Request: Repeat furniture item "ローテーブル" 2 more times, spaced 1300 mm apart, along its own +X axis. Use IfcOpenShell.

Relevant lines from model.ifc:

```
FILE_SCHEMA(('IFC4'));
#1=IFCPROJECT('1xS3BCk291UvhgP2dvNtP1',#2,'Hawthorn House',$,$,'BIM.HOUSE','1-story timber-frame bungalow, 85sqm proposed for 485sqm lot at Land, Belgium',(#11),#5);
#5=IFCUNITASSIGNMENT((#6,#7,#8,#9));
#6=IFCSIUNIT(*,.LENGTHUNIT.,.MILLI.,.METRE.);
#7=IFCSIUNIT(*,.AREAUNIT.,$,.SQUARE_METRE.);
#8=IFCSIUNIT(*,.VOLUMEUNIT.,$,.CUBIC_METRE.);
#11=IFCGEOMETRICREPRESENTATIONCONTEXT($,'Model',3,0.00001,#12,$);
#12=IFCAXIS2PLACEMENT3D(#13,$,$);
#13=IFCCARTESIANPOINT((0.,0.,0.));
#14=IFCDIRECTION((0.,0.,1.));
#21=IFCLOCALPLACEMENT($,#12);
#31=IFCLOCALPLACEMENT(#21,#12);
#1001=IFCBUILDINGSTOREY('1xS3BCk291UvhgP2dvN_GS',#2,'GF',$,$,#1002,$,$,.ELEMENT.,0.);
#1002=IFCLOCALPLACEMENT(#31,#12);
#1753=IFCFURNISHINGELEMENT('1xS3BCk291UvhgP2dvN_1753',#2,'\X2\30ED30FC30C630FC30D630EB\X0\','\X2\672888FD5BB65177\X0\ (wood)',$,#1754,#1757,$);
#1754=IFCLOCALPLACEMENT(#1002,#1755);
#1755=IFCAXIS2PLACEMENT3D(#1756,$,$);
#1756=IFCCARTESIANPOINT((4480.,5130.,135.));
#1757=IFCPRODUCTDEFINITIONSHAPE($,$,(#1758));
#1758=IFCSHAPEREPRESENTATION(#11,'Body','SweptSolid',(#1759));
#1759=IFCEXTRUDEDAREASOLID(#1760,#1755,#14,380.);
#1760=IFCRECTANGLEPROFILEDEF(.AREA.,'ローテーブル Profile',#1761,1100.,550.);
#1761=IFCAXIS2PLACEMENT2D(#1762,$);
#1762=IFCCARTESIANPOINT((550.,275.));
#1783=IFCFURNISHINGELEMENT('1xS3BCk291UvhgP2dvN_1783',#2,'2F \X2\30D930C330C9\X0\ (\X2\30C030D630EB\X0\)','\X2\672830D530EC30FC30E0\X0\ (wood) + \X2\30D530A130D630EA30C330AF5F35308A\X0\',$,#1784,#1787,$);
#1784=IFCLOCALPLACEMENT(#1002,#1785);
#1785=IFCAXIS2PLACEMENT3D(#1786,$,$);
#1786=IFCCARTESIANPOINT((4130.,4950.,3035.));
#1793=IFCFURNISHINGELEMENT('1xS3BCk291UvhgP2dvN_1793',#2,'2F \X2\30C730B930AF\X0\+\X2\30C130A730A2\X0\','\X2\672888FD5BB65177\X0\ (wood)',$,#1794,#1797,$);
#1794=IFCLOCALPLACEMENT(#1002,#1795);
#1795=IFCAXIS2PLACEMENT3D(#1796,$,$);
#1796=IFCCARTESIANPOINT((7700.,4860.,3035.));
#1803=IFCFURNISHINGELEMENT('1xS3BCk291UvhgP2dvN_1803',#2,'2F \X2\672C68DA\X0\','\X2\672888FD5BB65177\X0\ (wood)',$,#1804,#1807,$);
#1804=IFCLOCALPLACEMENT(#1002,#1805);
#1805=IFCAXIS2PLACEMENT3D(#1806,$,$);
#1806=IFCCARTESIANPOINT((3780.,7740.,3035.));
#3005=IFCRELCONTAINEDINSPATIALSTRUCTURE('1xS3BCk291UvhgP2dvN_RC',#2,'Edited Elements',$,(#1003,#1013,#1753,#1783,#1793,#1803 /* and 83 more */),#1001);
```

```python
import ifcopenshell
import ifcopenshell.api.geometry
import ifcopenshell.api.root
import ifcopenshell.util.element
import ifcopenshell.util.placement

model = ifcopenshell.open("model.ifc")


def reuse_history(source, copy):
    """copy_class also copies each property set's owner history, people and application; keep the originals."""
    for rel in copy.IsDefinedBy:
        if rel.is_a("IfcRelDefinesByProperties") and (history := rel.RelatingPropertyDefinition.OwnerHistory):
            rel.RelatingPropertyDefinition.OwnerHistory = source.OwnerHistory
            ifcopenshell.util.element.remove_deep2(model, history)


source = model.by_id(1753)
base = ifcopenshell.util.placement.get_local_placement(source.ObjectPlacement)
step = base[:3, 0] * 1300.0

for i in range(1, 3):
    copy = ifcopenshell.api.root.copy_class(model, product=source)
    copy.Representation = ifcopenshell.util.element.copy_deep(
        model, source.Representation, exclude=["IfcGeometricRepresentationContext", "IfcRepresentationMap"]
    )
    reuse_history(source, copy)
    matrix = base.copy()
    matrix[:3, 3] += i * step
    print("added at", matrix[:3, 3].round(3) + 0.0)
    ifcopenshell.api.geometry.edit_object_placement(model, product=copy, matrix=matrix, is_si=False)

model.write("model_v2.ifc")
```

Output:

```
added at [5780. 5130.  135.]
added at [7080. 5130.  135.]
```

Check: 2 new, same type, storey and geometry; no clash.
